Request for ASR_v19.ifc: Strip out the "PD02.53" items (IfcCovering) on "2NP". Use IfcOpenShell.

First a look at what the model holds.

```python
import ifcopenshell
import ifcopenshell.util.element

model = ifcopenshell.open("ASR_v19.ifc")
print(model.schema)
storey = next(s for s in model.by_type("IfcBuildingStorey") if s.Name == "2NP")
coverings = [e for e in ifcopenshell.util.element.get_decomposition(storey) if e.is_a("IfcCovering")]
seen = {}
for e in coverings:
    element_type = ifcopenshell.util.element.get_type(e)
    name = element_type.Name if element_type not in (None, e) else None
    seen[name] = seen.get(name, 0) + 1
for name, count in sorted(seen.items(), key=str):
    print(count, "x", name)
```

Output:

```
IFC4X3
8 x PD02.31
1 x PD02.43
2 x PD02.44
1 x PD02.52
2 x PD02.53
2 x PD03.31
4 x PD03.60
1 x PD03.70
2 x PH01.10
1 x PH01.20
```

```python
import ifcopenshell
import ifcopenshell.api.root
import ifcopenshell.util.element

model = ifcopenshell.open("ASR_v19.ifc")

storey = next(s for s in model.by_type("IfcBuildingStorey") if s.Name == "2NP")
coverings = [e for e in ifcopenshell.util.element.get_decomposition(storey) if e.is_a("IfcCovering")]
targets = [e for e in coverings if (t := ifcopenshell.util.element.get_type(e)) not in (None, e) and t.Name == "PD02.53"]

for e in targets:
    ifcopenshell.api.root.remove_product(model, product=e)
print(len(targets), "removed")

model.write("ASR_v19_updated.ifc")
```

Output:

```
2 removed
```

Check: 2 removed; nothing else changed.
